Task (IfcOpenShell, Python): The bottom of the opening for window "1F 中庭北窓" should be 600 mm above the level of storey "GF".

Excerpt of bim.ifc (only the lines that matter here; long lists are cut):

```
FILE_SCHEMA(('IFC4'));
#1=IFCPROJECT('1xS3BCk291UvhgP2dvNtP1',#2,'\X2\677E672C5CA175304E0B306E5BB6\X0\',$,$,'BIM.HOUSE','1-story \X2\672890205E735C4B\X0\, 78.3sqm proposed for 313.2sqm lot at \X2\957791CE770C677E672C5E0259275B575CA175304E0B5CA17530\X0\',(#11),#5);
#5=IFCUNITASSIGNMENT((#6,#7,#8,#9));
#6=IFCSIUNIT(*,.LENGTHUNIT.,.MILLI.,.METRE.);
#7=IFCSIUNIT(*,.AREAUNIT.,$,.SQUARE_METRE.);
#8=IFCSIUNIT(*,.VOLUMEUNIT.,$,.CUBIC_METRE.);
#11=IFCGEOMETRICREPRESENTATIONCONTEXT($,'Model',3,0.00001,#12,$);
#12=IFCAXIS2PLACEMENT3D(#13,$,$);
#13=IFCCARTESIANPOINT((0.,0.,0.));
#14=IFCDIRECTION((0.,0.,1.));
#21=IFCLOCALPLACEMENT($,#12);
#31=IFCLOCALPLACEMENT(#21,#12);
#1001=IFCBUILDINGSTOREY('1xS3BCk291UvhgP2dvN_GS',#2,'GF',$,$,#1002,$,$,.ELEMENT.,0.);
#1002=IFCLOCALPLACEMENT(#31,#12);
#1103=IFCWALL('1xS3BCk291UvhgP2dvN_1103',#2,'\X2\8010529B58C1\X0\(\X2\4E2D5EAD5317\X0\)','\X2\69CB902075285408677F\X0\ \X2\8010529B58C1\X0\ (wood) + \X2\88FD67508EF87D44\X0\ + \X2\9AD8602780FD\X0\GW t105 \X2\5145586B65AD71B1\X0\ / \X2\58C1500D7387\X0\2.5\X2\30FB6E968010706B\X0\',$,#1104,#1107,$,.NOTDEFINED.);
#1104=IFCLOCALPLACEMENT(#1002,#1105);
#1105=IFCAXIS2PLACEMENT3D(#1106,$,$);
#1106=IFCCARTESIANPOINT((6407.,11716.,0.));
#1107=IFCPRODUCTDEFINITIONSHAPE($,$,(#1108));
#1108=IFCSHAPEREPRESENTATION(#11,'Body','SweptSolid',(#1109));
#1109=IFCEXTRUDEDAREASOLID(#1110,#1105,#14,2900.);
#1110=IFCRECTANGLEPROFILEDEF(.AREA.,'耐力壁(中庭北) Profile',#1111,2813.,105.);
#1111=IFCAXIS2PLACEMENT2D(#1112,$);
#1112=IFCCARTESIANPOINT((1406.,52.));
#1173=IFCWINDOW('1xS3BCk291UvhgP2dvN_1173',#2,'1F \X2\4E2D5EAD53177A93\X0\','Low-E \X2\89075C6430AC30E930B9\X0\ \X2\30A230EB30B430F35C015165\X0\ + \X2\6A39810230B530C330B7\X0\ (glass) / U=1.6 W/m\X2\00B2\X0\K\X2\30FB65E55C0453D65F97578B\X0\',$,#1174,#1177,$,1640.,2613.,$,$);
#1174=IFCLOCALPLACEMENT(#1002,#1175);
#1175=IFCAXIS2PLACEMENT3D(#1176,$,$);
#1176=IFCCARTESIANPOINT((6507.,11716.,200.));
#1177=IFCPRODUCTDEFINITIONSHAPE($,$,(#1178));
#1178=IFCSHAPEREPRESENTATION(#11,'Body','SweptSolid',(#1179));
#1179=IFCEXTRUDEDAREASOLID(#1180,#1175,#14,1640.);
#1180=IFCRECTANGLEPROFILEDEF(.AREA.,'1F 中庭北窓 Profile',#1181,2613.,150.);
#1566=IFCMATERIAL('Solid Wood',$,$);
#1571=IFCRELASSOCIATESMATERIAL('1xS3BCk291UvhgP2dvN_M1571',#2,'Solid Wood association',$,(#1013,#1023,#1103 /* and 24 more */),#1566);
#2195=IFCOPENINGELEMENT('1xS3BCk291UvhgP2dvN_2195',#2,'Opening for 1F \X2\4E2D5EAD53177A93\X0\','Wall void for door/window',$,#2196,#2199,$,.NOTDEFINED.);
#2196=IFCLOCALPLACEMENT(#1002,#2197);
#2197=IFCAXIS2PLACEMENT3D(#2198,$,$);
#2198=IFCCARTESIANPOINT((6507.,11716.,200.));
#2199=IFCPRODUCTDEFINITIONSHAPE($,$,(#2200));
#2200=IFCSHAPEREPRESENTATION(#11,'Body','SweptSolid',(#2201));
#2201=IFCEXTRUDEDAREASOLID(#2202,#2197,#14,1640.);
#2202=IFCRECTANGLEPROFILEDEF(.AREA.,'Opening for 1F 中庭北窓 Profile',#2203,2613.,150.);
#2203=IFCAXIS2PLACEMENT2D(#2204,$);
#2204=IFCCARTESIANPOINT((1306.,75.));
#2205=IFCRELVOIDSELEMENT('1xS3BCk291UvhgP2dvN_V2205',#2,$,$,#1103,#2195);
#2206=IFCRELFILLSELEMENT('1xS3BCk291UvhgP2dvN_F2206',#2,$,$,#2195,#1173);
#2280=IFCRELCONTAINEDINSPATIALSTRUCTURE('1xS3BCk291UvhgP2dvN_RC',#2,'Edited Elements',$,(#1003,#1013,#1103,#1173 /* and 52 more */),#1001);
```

```python
import numpy as np
import ifcopenshell
import ifcopenshell.api.geometry
import ifcopenshell.geom
import ifcopenshell.util.element
import ifcopenshell.util.placement
import ifcopenshell.util.shape
import ifcopenshell.util.unit

model = ifcopenshell.open("bim.ifc")
unit_scale = ifcopenshell.util.unit.calculate_unit_scale(model)

window = model.by_guid("1xS3BCk291UvhgP2dvN_1173")
opening = window.FillsVoids[0].RelatingOpeningElement
storey = ifcopenshell.util.element.get_container(window, ifc_class="IfcBuildingStorey")
level = ifcopenshell.util.placement.get_local_placement(storey.ObjectPlacement)[2, 3]

# The opening's origin need not be at the sill, so measure its lowest point.
shape = ifcopenshell.geom.create_shape(ifcopenshell.geom.settings(), opening)
bottom = ifcopenshell.util.shape.get_shape_bottom_elevation(shape, shape.geometry) / unit_scale
dz = level + 600.0 - bottom

shift = np.array([0.0, 0.0, dz])
# The window is not placed relative to its opening, so move both.
for product in (opening, window):
    matrix = ifcopenshell.util.placement.get_local_placement(product.ObjectPlacement)
    matrix[:3, 3] += shift
    ifcopenshell.api.geometry.edit_object_placement(model, product=product, matrix=matrix, is_si=False)

print(f"moved by {dz * unit_scale:+.3f} m")

model.write("bim_updated.ifc")
```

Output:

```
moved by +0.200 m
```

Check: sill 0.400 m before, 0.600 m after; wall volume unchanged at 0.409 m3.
